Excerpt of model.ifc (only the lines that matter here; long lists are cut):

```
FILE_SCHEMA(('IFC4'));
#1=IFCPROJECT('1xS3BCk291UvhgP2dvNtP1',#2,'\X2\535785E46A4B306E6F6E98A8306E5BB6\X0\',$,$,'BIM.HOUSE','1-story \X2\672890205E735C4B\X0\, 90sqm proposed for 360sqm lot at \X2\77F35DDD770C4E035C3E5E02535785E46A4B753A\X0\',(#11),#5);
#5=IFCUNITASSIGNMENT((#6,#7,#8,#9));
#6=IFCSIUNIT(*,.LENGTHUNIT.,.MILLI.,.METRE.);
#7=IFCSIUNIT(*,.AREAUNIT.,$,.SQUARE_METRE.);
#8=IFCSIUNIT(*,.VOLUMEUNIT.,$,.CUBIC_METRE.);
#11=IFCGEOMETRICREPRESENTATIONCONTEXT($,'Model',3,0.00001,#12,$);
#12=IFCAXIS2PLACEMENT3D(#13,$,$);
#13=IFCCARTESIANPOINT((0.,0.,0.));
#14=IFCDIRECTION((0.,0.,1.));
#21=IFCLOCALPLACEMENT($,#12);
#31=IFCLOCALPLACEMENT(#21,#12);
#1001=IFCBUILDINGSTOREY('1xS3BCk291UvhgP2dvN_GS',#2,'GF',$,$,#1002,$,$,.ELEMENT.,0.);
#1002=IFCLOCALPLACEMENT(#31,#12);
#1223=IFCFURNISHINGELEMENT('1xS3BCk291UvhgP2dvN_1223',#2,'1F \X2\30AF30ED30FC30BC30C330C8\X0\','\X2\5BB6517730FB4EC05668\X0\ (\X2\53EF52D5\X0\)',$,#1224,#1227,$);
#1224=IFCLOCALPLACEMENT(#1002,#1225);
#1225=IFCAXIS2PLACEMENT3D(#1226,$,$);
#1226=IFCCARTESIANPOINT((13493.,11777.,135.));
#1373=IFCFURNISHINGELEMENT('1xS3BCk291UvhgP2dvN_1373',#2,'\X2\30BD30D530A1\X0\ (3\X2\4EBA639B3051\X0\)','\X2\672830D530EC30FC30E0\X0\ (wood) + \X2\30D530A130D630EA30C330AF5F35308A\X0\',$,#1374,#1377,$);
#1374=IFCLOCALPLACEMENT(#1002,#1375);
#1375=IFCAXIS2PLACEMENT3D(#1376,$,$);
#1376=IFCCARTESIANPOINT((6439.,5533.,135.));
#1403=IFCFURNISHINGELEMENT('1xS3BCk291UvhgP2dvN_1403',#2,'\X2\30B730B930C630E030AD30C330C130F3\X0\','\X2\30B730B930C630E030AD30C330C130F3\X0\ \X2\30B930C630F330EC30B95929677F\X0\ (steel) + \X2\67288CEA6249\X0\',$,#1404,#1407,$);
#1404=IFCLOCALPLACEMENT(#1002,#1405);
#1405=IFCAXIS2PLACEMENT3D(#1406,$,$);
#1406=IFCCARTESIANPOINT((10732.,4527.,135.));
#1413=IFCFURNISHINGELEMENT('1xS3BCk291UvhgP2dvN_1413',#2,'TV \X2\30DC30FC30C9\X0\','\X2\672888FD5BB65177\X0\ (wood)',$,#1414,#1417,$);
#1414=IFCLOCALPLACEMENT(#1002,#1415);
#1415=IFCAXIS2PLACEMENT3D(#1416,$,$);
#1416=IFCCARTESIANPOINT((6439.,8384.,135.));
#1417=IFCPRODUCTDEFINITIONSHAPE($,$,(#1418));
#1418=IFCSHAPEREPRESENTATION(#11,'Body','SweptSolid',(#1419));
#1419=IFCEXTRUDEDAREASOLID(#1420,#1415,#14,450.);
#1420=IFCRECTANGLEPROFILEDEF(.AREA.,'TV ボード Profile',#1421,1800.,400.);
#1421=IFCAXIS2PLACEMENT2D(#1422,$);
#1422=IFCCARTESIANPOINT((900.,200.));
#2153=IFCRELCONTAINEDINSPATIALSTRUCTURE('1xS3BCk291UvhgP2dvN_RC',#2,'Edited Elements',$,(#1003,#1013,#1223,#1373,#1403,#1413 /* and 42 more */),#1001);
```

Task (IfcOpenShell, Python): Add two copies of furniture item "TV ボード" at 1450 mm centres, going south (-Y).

```python
import numpy as np
import ifcopenshell
import ifcopenshell.api.geometry
import ifcopenshell.api.root
import ifcopenshell.util.element
import ifcopenshell.util.placement
import ifcopenshell.util.unit

model = ifcopenshell.open("model.ifc")
unit_scale = ifcopenshell.util.unit.calculate_unit_scale(model)


def reuse_history(source, copy):
    """copy_class also copies each property set's owner history, people and application; keep the originals."""
    for rel in copy.IsDefinedBy:
        if rel.is_a("IfcRelDefinesByProperties") and (history := rel.RelatingPropertyDefinition.OwnerHistory):
            rel.RelatingPropertyDefinition.OwnerHistory = source.OwnerHistory
            ifcopenshell.util.element.remove_deep2(model, history)


source = model.by_guid("1xS3BCk291UvhgP2dvN_1413")
base = ifcopenshell.util.placement.get_local_placement(source.ObjectPlacement)
step = np.array([0.0, -1.0, 0.0]) * 1.45 / unit_scale

for i in range(1, 3):
    copy = ifcopenshell.api.root.copy_class(model, product=source)
    copy.Representation = ifcopenshell.util.element.copy_deep(
        model, source.Representation, exclude=["IfcGeometricRepresentationContext", "IfcRepresentationMap"]
    )
    reuse_history(source, copy)
    matrix = base.copy()
    matrix[:3, 3] += i * step
    print("added at", matrix[:3, 3].round(3) + 0.0)
    ifcopenshell.api.geometry.edit_object_placement(model, product=copy, matrix=matrix, is_si=False)

model.write("model_rev.ifc")
```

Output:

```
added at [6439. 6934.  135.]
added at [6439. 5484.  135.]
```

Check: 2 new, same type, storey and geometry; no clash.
